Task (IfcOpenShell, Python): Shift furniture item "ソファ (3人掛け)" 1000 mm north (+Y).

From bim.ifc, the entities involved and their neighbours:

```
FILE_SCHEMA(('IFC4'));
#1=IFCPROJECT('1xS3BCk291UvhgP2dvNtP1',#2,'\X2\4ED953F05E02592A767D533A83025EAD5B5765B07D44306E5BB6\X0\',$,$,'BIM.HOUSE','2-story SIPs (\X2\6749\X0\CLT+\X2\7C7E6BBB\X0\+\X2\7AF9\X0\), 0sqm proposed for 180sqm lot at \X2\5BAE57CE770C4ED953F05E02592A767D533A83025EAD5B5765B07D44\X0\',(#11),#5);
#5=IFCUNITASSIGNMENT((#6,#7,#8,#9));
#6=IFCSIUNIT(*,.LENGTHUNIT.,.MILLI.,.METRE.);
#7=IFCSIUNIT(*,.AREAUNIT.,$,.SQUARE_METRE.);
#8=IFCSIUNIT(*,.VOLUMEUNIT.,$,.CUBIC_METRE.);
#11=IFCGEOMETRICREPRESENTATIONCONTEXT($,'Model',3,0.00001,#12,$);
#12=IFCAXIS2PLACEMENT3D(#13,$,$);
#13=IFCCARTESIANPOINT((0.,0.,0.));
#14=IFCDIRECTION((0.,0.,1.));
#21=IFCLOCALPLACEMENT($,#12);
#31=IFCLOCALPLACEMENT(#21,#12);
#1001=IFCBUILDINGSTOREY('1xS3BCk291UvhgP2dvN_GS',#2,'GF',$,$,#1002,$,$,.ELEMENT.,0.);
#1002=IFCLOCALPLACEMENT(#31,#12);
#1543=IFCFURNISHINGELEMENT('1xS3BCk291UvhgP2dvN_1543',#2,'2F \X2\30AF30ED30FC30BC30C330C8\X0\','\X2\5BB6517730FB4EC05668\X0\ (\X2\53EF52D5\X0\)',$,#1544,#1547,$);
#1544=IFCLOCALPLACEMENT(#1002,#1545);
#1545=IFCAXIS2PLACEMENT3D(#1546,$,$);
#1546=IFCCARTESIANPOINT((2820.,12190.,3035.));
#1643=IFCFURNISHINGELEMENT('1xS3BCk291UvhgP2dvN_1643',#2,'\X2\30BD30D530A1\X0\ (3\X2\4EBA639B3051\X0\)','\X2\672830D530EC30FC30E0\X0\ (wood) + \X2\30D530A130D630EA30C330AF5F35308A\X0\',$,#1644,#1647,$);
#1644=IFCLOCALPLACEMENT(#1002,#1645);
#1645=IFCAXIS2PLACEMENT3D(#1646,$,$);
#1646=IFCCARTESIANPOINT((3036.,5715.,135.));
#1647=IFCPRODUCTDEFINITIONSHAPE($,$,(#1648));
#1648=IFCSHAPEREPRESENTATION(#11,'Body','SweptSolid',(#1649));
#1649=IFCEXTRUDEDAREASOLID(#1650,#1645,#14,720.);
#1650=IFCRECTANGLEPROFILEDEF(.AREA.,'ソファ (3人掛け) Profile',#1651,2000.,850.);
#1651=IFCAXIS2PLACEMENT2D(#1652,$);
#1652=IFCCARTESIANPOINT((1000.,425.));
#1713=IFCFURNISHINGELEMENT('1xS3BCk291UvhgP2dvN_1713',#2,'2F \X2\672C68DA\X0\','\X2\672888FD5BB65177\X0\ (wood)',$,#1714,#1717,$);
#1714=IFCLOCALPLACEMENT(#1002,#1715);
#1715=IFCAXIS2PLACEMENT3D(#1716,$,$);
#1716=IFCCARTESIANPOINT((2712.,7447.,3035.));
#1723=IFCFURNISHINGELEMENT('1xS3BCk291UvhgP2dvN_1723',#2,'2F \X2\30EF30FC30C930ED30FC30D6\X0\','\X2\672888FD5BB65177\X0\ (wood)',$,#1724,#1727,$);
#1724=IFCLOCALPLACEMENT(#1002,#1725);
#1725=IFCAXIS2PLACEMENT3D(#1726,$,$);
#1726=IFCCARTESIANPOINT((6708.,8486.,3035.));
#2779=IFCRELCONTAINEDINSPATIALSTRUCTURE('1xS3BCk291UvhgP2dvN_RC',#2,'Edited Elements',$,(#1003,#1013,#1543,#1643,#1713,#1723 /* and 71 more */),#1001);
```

```python
import ifcopenshell
import ifcopenshell.api.geometry
import ifcopenshell.util.placement
import ifcopenshell.util.unit

model = ifcopenshell.open("bim.ifc")
unit_scale = ifcopenshell.util.unit.calculate_unit_scale(model)

item = model.by_id(1643)
matrix = ifcopenshell.util.placement.get_local_placement(item.ObjectPlacement)
matrix[1, 3] += 1 / unit_scale
ifcopenshell.api.geometry.edit_object_placement(model, product=item, matrix=matrix, is_si=False)

print(ifcopenshell.util.placement.get_local_placement(item.ObjectPlacement).round(3) + 0.0)

model.write("bim_edited.ifc")
```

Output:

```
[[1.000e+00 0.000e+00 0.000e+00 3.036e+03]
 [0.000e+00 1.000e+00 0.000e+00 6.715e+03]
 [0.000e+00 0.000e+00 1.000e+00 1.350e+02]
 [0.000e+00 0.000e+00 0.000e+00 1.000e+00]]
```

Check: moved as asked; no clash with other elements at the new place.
